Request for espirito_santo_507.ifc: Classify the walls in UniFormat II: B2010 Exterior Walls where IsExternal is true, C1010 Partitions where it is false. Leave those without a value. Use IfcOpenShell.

First a look at what the model holds.

```python
import ifcopenshell
import ifcopenshell.util.element

model = ifcopenshell.open("espirito_santo_507.ifc")
print(model.schema)
print("classifications:", [c.Name for c in model.by_type("IfcClassification")])
values = [ifcopenshell.util.element.get_pset(e, "Pset_WallCommon", "IsExternal") for e in model.by_type("IfcWall")]
for value in (True, False, None):
    print("IsExternal", value, values.count(value))
```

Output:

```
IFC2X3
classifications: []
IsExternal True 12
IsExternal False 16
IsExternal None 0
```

```python
import ifcopenshell
import ifcopenshell.api.classification
import ifcopenshell.util.element

model = ifcopenshell.open("espirito_santo_507.ifc")

# IFC2X3 requires Source and Edition and has no link from the project to the system.
system = model.create_entity("IfcClassification", Source="ASTM", Edition="E1557", Name="UniFormat II")

walls = model.by_type("IfcWall")
external = {e: ifcopenshell.util.element.get_pset(e, "Pset_WallCommon", "IsExternal") for e in walls}
for flag, code, name in ((True, "B2010", "Exterior Walls"), (False, "C1010", "Partitions")):
    products = [e for e in walls if external[e] is flag]
    ifcopenshell.api.classification.add_reference(
        model, products=products, classification=system, identification=code, name=name
    )
    print(code, len(products))

model.write("espirito_santo_507_rev.ifc")
```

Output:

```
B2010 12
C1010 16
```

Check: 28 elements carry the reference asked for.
